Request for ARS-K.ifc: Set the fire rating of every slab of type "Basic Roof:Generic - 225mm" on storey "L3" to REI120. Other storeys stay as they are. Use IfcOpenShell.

First a look at what the model holds.

```python
import ifcopenshell
import ifcopenshell.util.element

model = ifcopenshell.open("ARS-K.ifc")
print(model.schema)
storey = next(s for s in model.by_type("IfcBuildingStorey") if s.Name == "L3")
slabs = [e for e in ifcopenshell.util.element.get_decomposition(storey) if e.is_a("IfcSlab")]
seen = {}
for e in slabs:
    element_type = ifcopenshell.util.element.get_type(e)
    key = (element_type.Name if element_type != e and element_type else None, ifcopenshell.util.element.get_pset(e, "Pset_SlabCommon", "FireRating"))
    seen[key] = seen.get(key, 0) + 1
for (name, value), count in sorted(seen.items(), key=str):
    print(count, "x", name, "|", value)
```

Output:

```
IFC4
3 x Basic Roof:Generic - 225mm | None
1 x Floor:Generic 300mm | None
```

```python
import ifcopenshell
import ifcopenshell.api.pset
import ifcopenshell.util.element

model = ifcopenshell.open("ARS-K.ifc")

storey = next(s for s in model.by_type("IfcBuildingStorey") if s.Name == "L3")
slabs = [e for e in ifcopenshell.util.element.get_decomposition(storey) if e.is_a("IfcSlab")]

count = 0
for e in slabs:
    element_type = ifcopenshell.util.element.get_type(e)
    if element_type in (None, e) or element_type.Name != "Basic Roof:Generic - 225mm":
        continue
    # add_pset returns the element's existing set when there is one.
    pset = ifcopenshell.api.pset.add_pset(model, product=e, name="Pset_SlabCommon")
    ifcopenshell.api.pset.edit_pset(model, pset=pset, properties={"FireRating": "REI120"})
    count += 1

print(count, "slabs updated")

model.write("ARS-K_v2.ifc")
```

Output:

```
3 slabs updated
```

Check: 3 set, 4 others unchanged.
